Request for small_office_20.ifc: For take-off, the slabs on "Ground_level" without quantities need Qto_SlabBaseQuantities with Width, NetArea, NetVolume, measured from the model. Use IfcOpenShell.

First a look at what the model holds.

```python
import ifcopenshell
import ifcopenshell.util.element
import ifcopenshell.util.unit

model = ifcopenshell.open("small_office_20.ifc")
print(model.schema)
for unit_type in ("LENGTHUNIT", "AREAUNIT", "VOLUMEUNIT"):
    print(unit_type, ifcopenshell.util.unit.calculate_unit_scale(model, unit_type))
storey = next(s for s in model.by_type("IfcBuildingStorey") if s.Name == "Ground_level")
slabs = [e for e in ifcopenshell.util.element.get_decomposition(storey) if e.is_a("IfcSlab")]
for e in sorted(slabs, key=lambda e: e.id()):
    print(e.id(), e.is_a(), e.Name, list(ifcopenshell.util.element.get_psets(e, qtos_only=True)), sep=" | ")
```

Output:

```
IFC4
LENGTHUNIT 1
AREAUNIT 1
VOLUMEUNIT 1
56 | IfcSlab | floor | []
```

```python
import ifcopenshell
import ifcopenshell.api.pset
import ifcopenshell.geom
import ifcopenshell.util.element
import ifcopenshell.util.shape
import ifcopenshell.util.unit

model = ifcopenshell.open("small_office_20.ifc")
unit_scale = ifcopenshell.util.unit.calculate_unit_scale(model)
area_scale = ifcopenshell.util.unit.calculate_unit_scale(model, "AREAUNIT")
volume_scale = ifcopenshell.util.unit.calculate_unit_scale(model, "VOLUMEUNIT")
settings = ifcopenshell.geom.settings()

storey = next(s for s in model.by_type("IfcBuildingStorey") if s.Name == "Ground_level")
slabs = [e for e in ifcopenshell.util.element.get_decomposition(storey) if e.is_a("IfcSlab")]

for e in sorted(slabs, key=lambda e: e.id()):
    if ifcopenshell.util.element.get_psets(e, qtos_only=True, should_inherit=False):
        continue
    # Geometry comes back in metres, in the element's own axes.
    shape = ifcopenshell.geom.create_shape(settings, e)
    values = {
        "Width": ifcopenshell.util.shape.get_z(shape.geometry) / unit_scale,
        "NetArea": ifcopenshell.util.shape.get_footprint_area(shape.geometry) / area_scale,
        "NetVolume": ifcopenshell.util.shape.get_volume(shape.geometry) / volume_scale,
    }
    qto = ifcopenshell.api.pset.add_qto(model, product=e, name="Qto_SlabBaseQuantities")
    ifcopenshell.api.pset.edit_qto(model, qto=qto, properties=values)
    print(e.id(), {k: round(v, 3) for k, v in values.items()})

model.write("small_office_20-out.ifc")
```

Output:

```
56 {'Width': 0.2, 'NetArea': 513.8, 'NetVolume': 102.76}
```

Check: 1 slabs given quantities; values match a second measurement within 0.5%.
